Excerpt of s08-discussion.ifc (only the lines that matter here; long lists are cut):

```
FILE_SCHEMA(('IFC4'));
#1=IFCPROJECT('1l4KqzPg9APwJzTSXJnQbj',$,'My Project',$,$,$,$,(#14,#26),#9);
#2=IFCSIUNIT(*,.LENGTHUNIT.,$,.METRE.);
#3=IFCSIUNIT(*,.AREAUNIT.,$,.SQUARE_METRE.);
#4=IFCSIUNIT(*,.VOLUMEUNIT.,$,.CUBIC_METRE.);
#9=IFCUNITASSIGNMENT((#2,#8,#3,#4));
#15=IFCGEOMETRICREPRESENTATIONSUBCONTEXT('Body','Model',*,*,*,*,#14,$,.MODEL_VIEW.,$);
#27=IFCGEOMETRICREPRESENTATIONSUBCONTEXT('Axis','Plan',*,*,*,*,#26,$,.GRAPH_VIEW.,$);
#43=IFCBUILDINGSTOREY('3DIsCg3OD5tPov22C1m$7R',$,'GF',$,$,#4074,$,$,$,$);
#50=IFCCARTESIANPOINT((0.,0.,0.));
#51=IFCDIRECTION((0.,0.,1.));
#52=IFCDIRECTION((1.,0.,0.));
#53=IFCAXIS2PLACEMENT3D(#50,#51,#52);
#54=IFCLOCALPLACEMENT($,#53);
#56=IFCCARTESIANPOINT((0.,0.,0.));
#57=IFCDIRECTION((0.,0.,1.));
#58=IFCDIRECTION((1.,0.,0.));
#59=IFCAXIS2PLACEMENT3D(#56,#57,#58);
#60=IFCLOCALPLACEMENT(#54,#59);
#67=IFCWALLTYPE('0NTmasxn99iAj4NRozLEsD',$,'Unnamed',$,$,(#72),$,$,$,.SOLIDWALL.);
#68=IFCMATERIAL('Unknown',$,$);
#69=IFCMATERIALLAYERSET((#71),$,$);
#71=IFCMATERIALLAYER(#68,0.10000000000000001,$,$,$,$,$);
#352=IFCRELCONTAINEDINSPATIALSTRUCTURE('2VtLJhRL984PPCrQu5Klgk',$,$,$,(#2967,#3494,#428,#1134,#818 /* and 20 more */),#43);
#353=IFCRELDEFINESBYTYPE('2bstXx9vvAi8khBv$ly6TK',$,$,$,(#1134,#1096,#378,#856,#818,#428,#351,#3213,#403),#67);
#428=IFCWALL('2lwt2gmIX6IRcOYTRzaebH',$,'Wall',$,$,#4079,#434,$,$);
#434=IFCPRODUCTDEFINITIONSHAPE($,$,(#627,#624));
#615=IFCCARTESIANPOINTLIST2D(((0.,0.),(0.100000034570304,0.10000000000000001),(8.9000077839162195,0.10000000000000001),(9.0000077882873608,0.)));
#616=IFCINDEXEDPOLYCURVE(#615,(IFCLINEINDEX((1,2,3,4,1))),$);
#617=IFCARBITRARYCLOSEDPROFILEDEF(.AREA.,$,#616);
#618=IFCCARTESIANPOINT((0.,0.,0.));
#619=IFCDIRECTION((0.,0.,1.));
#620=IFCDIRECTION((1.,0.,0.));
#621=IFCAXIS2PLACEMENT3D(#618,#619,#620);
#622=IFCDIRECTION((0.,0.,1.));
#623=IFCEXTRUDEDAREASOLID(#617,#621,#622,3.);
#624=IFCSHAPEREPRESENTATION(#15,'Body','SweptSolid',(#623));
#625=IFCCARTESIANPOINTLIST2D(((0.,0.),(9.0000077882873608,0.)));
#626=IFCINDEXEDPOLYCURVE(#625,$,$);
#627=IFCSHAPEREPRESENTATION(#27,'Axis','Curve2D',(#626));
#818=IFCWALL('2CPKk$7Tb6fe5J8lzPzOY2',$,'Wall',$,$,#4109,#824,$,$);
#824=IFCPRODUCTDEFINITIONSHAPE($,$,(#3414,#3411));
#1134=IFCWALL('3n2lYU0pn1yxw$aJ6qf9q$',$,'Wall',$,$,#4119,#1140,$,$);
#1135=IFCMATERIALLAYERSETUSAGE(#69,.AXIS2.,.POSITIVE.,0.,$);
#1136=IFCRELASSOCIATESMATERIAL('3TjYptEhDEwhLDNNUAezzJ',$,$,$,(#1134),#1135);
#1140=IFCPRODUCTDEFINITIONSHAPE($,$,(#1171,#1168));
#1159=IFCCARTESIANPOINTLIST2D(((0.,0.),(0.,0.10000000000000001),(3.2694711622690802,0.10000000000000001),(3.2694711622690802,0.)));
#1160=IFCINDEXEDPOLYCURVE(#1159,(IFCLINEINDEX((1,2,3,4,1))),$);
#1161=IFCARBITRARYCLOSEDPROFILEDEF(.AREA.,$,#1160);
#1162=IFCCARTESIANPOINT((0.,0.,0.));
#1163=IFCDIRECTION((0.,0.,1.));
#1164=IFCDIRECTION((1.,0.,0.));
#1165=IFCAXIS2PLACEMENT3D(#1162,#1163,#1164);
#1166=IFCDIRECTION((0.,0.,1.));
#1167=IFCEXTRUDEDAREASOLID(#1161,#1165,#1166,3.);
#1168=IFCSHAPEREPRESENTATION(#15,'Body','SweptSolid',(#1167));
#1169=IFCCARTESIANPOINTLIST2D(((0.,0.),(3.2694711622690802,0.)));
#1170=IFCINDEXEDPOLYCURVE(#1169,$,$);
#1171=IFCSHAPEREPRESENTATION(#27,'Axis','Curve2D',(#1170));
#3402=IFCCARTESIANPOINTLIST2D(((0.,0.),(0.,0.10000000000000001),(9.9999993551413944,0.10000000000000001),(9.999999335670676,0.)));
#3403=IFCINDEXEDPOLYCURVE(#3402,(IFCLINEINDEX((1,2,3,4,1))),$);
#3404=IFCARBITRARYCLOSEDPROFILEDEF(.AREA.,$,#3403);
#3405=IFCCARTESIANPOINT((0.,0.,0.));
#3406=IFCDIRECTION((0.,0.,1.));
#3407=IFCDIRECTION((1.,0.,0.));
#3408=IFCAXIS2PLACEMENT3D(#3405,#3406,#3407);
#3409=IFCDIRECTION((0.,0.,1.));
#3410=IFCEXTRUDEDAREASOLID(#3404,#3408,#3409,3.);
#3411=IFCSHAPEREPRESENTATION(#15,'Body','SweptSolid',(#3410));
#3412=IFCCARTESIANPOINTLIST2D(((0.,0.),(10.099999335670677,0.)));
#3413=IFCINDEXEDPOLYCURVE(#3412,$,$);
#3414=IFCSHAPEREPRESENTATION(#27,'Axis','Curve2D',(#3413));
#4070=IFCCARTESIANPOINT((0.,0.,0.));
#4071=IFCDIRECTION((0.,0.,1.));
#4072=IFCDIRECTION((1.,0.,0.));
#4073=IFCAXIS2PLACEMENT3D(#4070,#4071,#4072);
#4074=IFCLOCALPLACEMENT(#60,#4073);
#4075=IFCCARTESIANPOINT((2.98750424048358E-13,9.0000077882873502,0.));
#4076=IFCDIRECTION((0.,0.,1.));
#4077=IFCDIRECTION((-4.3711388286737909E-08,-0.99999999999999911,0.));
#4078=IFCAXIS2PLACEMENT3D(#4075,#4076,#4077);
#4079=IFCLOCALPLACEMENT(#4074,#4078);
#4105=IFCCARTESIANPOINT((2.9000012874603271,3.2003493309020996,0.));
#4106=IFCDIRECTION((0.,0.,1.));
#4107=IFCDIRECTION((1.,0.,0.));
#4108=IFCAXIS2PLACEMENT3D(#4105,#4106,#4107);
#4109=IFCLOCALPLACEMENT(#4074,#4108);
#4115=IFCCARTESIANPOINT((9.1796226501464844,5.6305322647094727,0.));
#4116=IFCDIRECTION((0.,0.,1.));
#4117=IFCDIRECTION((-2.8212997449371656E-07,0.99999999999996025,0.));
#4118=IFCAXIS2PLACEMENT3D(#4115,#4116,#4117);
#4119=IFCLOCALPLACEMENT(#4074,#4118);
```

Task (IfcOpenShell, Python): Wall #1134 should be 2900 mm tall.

```python
import ifcopenshell
import ifcopenshell.geom
import ifcopenshell.util.representation
import ifcopenshell.util.shape
import ifcopenshell.util.unit

model = ifcopenshell.open("s08-discussion.ifc")
unit_scale = ifcopenshell.util.unit.calculate_unit_scale(model)
settings = ifcopenshell.geom.settings()


def volume(element):
    """Net volume in cubic metres, openings subtracted."""
    shape = ifcopenshell.geom.create_shape(settings, element)
    return ifcopenshell.util.shape.get_volume(shape.geometry)


wall = model.by_guid("3n2lYU0pn1yxw$aJ6qf9q$")
before = volume(wall)

body = ifcopenshell.util.representation.get_representation(wall, "Model", "Body")
solid = body.Items[0]
old_height = solid.Depth
solid.Depth = 2.9 / unit_scale
after = volume(wall)

print(f"height {old_height:g} -> {solid.Depth:g}, volume {before:.3f} -> {after:.3f} m3")

model.write("s08-discussion_edited.ifc")
```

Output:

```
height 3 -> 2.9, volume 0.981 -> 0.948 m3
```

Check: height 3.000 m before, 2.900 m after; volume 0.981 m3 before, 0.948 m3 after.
